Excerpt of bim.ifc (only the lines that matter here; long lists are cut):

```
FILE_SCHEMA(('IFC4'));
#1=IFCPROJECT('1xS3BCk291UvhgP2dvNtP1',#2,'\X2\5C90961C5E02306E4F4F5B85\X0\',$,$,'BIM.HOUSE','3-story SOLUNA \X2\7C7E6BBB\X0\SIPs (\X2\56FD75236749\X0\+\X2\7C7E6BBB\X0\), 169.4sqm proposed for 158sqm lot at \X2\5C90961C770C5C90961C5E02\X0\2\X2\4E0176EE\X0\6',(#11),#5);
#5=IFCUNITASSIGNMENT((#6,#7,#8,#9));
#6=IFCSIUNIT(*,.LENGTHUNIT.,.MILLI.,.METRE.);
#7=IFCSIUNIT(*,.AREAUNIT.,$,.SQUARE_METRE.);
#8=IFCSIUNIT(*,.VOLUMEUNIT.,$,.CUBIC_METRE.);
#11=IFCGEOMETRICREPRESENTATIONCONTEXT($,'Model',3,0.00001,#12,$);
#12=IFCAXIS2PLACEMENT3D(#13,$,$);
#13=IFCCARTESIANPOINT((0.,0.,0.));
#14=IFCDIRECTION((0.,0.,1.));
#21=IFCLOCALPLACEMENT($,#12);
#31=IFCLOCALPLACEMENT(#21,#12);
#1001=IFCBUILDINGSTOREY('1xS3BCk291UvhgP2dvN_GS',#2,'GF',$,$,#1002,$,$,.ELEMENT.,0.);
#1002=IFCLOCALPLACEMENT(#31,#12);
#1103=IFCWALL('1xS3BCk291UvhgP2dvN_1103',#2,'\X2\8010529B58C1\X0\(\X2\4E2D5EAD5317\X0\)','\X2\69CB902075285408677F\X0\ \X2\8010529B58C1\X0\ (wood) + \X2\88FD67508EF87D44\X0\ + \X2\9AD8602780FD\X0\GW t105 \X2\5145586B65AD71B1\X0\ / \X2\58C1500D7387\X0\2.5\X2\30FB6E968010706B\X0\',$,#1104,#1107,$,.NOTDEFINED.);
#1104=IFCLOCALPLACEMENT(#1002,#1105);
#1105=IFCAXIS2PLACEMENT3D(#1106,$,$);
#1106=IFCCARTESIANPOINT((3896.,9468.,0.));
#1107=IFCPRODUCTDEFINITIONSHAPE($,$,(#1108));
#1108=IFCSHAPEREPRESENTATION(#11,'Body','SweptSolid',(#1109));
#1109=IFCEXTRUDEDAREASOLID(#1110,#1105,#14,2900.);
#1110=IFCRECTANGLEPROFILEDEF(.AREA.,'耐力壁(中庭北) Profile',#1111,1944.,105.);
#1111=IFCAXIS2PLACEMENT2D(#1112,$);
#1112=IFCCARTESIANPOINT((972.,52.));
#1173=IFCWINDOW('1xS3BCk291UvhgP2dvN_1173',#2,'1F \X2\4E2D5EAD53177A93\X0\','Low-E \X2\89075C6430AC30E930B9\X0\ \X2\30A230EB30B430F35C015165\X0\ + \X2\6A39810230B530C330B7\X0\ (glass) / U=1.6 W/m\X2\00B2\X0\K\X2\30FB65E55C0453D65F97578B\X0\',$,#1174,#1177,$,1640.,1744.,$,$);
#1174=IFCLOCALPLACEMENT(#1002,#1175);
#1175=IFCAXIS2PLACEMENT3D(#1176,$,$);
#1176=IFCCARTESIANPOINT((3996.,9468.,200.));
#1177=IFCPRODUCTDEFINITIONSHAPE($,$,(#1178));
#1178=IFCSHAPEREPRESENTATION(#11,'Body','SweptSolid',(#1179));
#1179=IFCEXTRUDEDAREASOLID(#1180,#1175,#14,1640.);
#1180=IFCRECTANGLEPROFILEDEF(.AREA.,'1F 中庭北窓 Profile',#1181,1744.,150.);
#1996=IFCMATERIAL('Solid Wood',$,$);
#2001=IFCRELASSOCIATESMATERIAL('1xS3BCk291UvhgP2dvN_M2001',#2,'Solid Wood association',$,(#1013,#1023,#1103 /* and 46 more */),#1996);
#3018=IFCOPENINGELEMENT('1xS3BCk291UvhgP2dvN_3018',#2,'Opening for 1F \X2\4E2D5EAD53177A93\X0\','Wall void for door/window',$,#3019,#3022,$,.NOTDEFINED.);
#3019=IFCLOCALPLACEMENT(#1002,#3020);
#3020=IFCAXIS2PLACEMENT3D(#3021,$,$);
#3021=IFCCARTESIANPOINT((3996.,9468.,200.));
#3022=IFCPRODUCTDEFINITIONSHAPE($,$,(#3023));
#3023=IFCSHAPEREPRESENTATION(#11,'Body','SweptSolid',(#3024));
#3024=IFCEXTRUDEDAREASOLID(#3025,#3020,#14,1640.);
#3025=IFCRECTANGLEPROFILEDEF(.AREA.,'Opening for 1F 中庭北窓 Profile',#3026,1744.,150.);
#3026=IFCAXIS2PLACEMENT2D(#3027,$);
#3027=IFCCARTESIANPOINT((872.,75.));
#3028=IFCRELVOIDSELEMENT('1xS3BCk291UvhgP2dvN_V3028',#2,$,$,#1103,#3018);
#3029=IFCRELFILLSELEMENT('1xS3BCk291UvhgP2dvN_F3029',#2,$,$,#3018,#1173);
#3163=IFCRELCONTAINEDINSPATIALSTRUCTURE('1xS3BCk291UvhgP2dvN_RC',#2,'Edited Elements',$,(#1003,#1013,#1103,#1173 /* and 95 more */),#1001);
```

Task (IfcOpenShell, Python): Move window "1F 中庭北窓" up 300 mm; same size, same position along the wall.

```python
import numpy as np
import ifcopenshell
import ifcopenshell.api.geometry
import ifcopenshell.util.placement
import ifcopenshell.util.unit

model = ifcopenshell.open("bim.ifc")
unit_scale = ifcopenshell.util.unit.calculate_unit_scale(model)

window = model.by_guid("1xS3BCk291UvhgP2dvN_1173")
opening = window.FillsVoids[0].RelatingOpeningElement
dz = 300.0

shift = np.array([0.0, 0.0, dz])
# The window is not placed relative to its opening, so move both.
for product in (opening, window):
    matrix = ifcopenshell.util.placement.get_local_placement(product.ObjectPlacement)
    matrix[:3, 3] += shift
    ifcopenshell.api.geometry.edit_object_placement(model, product=product, matrix=matrix, is_si=False)

print(f"moved by {dz * unit_scale:+.3f} m")

model.write("bim_edited.ifc")
```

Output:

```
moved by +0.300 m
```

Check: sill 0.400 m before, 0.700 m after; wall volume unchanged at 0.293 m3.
